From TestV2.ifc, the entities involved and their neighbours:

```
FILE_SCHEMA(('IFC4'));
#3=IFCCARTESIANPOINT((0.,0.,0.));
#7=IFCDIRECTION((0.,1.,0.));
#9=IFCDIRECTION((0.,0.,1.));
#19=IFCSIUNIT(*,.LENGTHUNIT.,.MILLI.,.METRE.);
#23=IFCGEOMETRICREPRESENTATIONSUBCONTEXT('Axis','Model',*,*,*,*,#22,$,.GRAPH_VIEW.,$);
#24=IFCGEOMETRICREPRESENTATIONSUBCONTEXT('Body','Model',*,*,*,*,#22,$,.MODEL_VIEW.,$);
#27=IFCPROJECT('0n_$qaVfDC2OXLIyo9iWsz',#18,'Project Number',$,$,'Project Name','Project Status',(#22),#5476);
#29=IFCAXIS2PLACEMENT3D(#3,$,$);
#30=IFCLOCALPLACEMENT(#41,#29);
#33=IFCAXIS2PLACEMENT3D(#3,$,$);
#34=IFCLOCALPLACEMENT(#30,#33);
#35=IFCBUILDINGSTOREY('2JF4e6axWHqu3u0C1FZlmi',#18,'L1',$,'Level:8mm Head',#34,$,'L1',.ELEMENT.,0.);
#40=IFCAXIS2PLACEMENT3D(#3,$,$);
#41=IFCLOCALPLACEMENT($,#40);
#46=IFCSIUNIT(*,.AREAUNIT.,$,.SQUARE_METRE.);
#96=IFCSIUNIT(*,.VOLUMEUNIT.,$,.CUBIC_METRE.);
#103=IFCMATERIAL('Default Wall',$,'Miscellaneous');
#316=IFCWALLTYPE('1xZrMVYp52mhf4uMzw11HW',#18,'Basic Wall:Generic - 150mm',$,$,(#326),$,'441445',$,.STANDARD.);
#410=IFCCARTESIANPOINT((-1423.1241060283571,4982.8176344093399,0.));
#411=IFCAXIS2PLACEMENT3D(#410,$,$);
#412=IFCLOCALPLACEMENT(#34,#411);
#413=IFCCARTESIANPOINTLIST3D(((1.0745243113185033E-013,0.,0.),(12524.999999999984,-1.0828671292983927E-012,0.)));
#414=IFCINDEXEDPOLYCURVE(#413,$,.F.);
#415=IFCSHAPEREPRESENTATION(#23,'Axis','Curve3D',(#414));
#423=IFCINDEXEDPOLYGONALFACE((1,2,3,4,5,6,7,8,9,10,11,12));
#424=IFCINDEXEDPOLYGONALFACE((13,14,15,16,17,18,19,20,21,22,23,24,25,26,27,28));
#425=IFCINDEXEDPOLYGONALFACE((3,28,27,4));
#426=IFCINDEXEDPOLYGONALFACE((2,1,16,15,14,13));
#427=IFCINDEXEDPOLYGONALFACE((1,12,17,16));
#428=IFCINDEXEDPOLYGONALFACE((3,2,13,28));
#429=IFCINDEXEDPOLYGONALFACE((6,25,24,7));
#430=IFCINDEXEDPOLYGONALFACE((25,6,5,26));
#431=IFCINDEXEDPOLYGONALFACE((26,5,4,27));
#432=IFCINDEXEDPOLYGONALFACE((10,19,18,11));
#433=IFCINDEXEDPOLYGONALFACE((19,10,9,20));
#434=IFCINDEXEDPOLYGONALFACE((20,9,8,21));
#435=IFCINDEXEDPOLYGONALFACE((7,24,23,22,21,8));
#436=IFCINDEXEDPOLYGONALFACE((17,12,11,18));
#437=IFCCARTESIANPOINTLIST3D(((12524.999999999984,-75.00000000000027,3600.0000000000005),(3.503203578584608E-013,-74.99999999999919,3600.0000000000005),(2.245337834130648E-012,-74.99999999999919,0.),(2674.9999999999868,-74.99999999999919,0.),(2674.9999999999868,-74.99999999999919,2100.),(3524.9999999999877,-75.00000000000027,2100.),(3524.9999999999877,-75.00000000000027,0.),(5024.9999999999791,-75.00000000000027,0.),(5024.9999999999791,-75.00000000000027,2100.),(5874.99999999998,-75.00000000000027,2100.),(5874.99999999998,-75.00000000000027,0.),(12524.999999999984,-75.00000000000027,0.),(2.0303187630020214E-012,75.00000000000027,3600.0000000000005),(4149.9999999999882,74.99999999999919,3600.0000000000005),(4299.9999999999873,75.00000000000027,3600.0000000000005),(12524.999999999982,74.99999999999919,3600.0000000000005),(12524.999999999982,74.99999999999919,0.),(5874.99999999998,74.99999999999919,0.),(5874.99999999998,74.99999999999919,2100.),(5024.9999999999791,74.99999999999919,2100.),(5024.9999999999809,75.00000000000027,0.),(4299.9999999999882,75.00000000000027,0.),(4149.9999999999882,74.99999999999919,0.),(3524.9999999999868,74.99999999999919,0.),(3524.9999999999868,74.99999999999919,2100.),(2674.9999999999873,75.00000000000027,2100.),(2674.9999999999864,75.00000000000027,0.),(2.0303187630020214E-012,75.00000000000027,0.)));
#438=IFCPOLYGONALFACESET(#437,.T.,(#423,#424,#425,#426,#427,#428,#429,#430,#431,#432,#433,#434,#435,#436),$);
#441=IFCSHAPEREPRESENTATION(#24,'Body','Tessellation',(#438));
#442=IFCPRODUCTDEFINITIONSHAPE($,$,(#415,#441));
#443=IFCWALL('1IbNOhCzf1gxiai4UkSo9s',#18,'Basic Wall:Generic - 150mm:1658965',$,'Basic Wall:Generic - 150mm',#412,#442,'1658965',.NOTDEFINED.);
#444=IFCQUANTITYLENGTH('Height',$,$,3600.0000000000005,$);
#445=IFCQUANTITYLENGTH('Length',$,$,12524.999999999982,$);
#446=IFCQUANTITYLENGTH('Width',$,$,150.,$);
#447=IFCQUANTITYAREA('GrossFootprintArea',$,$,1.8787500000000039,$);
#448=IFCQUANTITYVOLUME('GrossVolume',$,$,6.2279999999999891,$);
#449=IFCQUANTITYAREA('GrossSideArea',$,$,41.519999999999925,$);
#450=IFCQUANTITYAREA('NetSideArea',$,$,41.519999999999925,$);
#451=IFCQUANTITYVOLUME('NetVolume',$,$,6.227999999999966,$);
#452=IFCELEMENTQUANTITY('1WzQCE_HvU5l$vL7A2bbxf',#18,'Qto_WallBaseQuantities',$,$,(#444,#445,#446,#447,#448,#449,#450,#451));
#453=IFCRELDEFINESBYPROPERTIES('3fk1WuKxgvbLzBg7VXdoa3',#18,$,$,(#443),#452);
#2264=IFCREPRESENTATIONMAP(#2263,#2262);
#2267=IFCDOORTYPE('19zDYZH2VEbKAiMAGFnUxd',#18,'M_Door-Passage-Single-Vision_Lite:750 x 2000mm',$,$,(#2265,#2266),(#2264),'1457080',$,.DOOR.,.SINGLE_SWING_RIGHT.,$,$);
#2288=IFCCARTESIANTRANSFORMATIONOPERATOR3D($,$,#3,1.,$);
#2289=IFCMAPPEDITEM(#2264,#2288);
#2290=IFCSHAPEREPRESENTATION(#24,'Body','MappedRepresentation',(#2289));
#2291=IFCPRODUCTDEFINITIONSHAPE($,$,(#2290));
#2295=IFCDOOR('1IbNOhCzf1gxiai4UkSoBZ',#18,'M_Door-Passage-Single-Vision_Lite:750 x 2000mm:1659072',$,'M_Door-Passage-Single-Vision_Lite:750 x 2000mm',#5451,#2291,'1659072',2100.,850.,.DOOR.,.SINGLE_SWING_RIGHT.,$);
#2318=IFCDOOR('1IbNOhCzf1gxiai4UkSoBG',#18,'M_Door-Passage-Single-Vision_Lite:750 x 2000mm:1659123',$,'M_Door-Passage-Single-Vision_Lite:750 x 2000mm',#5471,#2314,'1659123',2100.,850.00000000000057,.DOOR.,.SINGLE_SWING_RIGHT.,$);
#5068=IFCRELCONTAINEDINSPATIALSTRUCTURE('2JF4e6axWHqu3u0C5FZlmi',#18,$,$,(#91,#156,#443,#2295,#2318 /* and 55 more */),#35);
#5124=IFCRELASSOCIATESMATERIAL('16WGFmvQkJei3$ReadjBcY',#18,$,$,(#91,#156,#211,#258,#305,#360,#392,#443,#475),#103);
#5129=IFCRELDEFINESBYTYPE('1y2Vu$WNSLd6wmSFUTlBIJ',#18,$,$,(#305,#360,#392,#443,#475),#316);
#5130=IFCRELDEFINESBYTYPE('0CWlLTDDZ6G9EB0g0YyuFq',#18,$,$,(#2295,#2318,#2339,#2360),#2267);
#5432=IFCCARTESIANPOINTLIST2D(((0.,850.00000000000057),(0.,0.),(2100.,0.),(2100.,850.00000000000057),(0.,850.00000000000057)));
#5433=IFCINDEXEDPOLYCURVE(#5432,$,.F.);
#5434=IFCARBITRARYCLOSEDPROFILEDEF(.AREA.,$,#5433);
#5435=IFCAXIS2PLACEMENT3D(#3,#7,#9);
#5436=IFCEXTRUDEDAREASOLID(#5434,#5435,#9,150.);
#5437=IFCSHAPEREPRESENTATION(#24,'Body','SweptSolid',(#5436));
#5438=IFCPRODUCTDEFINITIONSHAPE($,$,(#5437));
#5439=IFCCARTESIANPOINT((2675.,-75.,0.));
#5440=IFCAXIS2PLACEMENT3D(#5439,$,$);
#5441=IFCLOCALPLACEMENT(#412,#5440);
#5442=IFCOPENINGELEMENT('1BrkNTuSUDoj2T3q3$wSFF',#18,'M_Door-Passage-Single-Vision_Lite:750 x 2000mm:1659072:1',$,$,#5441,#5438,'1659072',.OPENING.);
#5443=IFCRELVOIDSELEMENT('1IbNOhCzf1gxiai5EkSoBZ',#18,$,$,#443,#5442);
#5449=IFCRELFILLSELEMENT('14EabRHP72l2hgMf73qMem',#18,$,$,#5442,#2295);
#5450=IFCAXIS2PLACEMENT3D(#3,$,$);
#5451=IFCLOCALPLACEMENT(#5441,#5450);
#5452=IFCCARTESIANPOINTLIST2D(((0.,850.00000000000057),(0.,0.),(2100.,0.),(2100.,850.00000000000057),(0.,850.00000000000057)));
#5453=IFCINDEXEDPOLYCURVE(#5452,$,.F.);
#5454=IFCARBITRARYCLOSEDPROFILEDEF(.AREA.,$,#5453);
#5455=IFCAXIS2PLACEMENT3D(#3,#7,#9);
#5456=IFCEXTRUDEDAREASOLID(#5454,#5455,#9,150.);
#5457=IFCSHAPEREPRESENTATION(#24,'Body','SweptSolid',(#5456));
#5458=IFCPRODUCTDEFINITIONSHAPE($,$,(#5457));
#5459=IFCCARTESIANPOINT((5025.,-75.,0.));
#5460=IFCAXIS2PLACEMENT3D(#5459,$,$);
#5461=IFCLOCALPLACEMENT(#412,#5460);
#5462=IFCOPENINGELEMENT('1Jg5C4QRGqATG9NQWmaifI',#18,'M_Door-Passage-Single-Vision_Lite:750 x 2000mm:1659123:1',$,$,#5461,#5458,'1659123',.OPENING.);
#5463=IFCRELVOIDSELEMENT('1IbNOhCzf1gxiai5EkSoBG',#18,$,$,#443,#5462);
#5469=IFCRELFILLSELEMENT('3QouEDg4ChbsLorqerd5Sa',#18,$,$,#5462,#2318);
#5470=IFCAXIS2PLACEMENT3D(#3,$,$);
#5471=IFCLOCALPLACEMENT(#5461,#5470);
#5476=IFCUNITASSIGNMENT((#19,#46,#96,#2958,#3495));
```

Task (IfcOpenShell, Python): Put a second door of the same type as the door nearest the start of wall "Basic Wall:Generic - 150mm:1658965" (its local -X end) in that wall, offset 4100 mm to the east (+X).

```python
import ifcopenshell
import ifcopenshell.api.feature
import ifcopenshell.api.geometry
import ifcopenshell.api.pset
import ifcopenshell.api.root
import ifcopenshell.geom
import ifcopenshell.util.element
import ifcopenshell.util.placement
import ifcopenshell.util.shape
import ifcopenshell.util.unit

model = ifcopenshell.open("TestV2.ifc")
unit_scale = ifcopenshell.util.unit.calculate_unit_scale(model)
area_scale = ifcopenshell.util.unit.calculate_unit_scale(model, "AREAUNIT")
volume_scale = ifcopenshell.util.unit.calculate_unit_scale(model, "VOLUMEUNIT")
settings = ifcopenshell.geom.settings()


def volume(element):
    """Net volume in cubic metres, openings subtracted."""
    shape = ifcopenshell.geom.create_shape(settings, element)
    return ifcopenshell.util.shape.get_volume(shape.geometry)


def reuse_history(source, copy):
    """copy_class also copies each property set's owner history, people and application; keep the originals."""
    for rel in copy.IsDefinedBy:
        if rel.is_a("IfcRelDefinesByProperties") and (history := rel.RelatingPropertyDefinition.OwnerHistory):
            rel.RelatingPropertyDefinition.OwnerHistory = source.OwnerHistory
            ifcopenshell.util.element.remove_deep2(model, history)


door = model.by_guid("1IbNOhCzf1gxiai4UkSoBZ")
opening = door.FillsVoids[0].RelatingOpeningElement
wall = opening.VoidsElements[0].RelatingBuildingElement
before = volume(wall)
shift = ifcopenshell.util.placement.get_local_placement(wall.ObjectPlacement)[:3, 0] * 4.1 / unit_scale

# copy_class copies the void relationship, type, container and properties, but no geometry.
new_opening = ifcopenshell.api.root.copy_class(model, product=opening)
new_opening.Representation = ifcopenshell.util.element.copy_deep(
    model, opening.Representation, exclude=["IfcGeometricRepresentationContext", "IfcRepresentationMap"]
)
new_opening.Name = "M_Door-Passage-Single-Vision_Lite:750 x 2000mm"
new_opening.Tag = None
reuse_history(opening, new_opening)
new_door = ifcopenshell.api.root.copy_class(model, product=door)
new_door.Representation = ifcopenshell.util.element.copy_deep(
    model, door.Representation, exclude=["IfcGeometricRepresentationContext", "IfcRepresentationMap"]
)
new_door.Name = "M_Door-Passage-Single-Vision_Lite:750 x 2000mm"
new_door.Tag = None
reuse_history(door, new_door)
ifcopenshell.api.feature.add_filling(model, opening=new_opening, element=new_door)

for old, new in ((opening, new_opening), (door, new_door)):
    matrix = ifcopenshell.util.placement.get_local_placement(old.ObjectPlacement)
    matrix[:3, 3] += shift
    ifcopenshell.api.geometry.edit_object_placement(model, product=new, matrix=matrix, is_si=False)

after = volume(wall)
thickness = 0.15  # wall thickness in metres

# Update the wall's stored quantities.
qto = model.by_id(ifcopenshell.util.element.get_pset(wall, "Qto_WallBaseQuantities", should_inherit=False)["id"])
ifcopenshell.api.pset.edit_qto(model, qto=qto, properties={
    "NetSideArea": after / thickness / area_scale,
    "NetVolume": after / volume_scale,
})

print(f"wall volume {before:.3f} -> {after:.3f} m3")

model.write("TestV2_v2.ifc")
```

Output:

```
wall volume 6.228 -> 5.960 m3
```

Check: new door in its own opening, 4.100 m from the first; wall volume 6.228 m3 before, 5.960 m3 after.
